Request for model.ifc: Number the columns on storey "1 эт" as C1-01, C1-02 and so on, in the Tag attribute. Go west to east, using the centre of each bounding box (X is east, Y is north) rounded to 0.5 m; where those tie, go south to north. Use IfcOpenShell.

First a look at what the model holds.

```python
import ifcopenshell
import ifcopenshell.util.element
import ifcopenshell.util.placement

model = ifcopenshell.open("model.ifc")
print(model.schema)
storey = next(s for s in model.by_type("IfcBuildingStorey") if s.Name == "1 эт")
columns = [e for e in ifcopenshell.util.element.get_decomposition(storey) if e.is_a("IfcColumn")]
for e in sorted(columns, key=lambda e: e.id()):
    origin = ifcopenshell.util.placement.get_local_placement(e.ObjectPlacement)[:3, 3]
    print(e.id(), e.Tag, e.Name, origin.round(2) + 0.0, sep=" | ")
```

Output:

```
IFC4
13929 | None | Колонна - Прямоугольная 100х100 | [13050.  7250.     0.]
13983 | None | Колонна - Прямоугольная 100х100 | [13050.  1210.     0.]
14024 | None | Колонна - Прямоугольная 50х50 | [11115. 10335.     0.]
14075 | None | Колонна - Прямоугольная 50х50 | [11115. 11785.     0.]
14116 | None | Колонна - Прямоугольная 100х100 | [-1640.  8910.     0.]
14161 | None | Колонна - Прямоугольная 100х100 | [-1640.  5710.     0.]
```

```python
import ifcopenshell
import ifcopenshell.geom
import ifcopenshell.util.element
import ifcopenshell.util.shape

model = ifcopenshell.open("model.ifc")
settings = ifcopenshell.geom.settings()
settings.set("use-world-coords", True)


def centre(element):
    shape = ifcopenshell.geom.create_shape(settings, element)
    return ifcopenshell.util.shape.get_bbox_centroid(shape.geometry)


storey = next(s for s in model.by_type("IfcBuildingStorey") if s.Name == "1 эт")
columns = [e for e in ifcopenshell.util.element.get_decomposition(storey) if e.is_a("IfcColumn")]

# Insertion points can sit at a corner or the storey origin, so sort by the geometry (in metres).
centres = {e: centre(e) for e in columns}
columns.sort(key=lambda e: (round(centres[e][0] / 0.5), centres[e][1]))

for i, e in enumerate(columns, start=1):
    number = f"C1-{i:02d}"
    e.Tag = number
    print(e.id(), number)

model.write("model_updated.ifc")
```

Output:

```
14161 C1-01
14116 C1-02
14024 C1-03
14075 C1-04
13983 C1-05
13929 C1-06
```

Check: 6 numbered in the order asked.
